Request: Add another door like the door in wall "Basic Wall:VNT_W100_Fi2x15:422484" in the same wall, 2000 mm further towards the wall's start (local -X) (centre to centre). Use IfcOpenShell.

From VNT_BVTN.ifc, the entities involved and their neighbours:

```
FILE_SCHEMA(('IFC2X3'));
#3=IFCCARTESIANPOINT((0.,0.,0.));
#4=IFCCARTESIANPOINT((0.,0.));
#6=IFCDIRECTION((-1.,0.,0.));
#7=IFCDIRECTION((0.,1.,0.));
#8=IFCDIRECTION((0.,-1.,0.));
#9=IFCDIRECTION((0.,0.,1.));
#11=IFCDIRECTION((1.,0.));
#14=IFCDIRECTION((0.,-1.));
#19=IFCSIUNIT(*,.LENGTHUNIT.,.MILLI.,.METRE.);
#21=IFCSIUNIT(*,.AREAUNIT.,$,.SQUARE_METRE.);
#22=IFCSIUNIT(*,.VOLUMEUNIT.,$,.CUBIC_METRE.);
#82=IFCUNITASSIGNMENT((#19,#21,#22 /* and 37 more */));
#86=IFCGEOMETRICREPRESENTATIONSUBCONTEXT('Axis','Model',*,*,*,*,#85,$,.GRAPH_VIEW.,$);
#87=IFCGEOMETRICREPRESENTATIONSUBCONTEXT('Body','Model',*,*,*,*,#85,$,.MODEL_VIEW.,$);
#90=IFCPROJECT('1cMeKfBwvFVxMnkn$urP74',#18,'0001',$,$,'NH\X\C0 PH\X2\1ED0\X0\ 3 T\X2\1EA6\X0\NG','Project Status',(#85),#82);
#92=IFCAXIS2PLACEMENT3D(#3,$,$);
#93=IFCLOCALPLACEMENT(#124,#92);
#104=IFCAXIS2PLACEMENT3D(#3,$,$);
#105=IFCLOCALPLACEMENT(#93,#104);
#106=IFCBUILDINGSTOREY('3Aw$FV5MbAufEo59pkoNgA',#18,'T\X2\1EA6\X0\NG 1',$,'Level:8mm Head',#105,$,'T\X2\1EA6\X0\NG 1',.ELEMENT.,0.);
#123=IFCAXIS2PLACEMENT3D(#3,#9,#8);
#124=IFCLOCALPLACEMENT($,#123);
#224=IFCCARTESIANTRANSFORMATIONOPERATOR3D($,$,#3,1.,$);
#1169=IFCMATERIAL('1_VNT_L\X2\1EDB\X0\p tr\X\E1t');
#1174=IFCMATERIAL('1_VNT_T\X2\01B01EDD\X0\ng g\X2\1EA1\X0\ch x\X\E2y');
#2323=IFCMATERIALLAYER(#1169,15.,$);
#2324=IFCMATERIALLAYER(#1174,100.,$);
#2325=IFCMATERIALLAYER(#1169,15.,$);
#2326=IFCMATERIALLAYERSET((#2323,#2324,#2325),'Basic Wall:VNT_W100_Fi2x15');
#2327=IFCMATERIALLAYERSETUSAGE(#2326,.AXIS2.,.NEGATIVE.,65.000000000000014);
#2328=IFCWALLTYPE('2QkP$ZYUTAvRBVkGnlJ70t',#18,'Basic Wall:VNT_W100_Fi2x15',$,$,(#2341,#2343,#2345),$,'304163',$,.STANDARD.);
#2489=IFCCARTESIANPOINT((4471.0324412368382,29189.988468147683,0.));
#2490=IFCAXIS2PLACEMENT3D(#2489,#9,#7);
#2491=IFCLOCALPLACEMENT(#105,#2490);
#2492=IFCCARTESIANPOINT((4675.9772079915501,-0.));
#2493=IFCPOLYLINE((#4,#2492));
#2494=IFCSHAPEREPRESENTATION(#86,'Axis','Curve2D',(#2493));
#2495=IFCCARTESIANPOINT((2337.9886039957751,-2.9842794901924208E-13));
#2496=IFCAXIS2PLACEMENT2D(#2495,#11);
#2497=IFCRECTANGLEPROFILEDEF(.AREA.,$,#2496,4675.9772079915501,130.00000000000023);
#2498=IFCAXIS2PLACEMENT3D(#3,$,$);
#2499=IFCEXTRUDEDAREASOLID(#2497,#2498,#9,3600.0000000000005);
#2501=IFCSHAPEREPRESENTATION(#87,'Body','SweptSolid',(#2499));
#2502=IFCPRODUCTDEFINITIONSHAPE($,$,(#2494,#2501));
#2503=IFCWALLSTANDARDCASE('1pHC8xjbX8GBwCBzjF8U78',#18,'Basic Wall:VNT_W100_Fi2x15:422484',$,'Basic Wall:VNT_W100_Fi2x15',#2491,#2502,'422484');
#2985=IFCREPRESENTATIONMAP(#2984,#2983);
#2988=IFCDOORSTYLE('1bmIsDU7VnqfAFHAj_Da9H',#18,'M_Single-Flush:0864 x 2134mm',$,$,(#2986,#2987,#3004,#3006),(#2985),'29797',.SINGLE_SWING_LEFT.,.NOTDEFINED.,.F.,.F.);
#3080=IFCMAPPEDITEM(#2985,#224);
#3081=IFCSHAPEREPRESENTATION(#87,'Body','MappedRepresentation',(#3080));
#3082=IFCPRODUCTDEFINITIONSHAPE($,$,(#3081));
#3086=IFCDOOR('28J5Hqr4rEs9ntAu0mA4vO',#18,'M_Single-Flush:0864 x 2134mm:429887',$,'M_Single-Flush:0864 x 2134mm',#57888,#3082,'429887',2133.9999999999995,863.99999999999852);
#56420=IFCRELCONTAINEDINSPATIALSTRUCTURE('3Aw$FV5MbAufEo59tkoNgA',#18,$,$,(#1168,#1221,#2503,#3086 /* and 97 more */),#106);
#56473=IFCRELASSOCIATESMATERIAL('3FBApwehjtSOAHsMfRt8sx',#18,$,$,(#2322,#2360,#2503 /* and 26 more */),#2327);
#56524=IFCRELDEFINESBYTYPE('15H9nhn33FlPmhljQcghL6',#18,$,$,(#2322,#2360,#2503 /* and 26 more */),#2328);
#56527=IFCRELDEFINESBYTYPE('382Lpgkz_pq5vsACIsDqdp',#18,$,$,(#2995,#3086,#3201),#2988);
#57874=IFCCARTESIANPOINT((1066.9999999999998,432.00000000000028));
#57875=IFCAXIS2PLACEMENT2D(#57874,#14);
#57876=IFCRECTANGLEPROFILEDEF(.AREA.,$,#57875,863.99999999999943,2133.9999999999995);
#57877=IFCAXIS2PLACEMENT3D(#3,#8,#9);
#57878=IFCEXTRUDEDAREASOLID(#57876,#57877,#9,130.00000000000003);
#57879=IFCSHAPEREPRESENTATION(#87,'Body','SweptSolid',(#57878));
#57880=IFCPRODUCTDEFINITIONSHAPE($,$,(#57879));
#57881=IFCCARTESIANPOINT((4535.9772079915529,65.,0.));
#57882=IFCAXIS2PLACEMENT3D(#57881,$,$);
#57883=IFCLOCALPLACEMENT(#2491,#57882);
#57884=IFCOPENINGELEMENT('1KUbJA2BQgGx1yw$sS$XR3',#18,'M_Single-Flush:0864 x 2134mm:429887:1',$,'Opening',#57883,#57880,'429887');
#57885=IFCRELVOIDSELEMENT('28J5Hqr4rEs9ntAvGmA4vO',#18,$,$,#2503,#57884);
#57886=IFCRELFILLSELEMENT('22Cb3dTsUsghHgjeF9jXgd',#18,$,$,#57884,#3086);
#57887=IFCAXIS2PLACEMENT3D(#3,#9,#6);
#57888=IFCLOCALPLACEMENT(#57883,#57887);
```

```python
import ifcopenshell
import ifcopenshell.api.feature
import ifcopenshell.api.geometry
import ifcopenshell.api.root
import ifcopenshell.geom
import ifcopenshell.util.element
import ifcopenshell.util.placement
import ifcopenshell.util.shape

model = ifcopenshell.open("VNT_BVTN.ifc")
settings = ifcopenshell.geom.settings()


def volume(element):
    """Net volume in cubic metres, openings subtracted."""
    shape = ifcopenshell.geom.create_shape(settings, element)
    return ifcopenshell.util.shape.get_volume(shape.geometry)


def reuse_history(source, copy):
    """copy_class also copies each property set's owner history, people and application; keep the originals."""
    for rel in copy.IsDefinedBy:
        if rel.is_a("IfcRelDefinesByProperties") and (history := rel.RelatingPropertyDefinition.OwnerHistory):
            rel.RelatingPropertyDefinition.OwnerHistory = source.OwnerHistory
            ifcopenshell.util.element.remove_deep2(model, history)


door = model.by_guid("28J5Hqr4rEs9ntAu0mA4vO")
opening = door.FillsVoids[0].RelatingOpeningElement
wall = opening.VoidsElements[0].RelatingBuildingElement
before = volume(wall)
shift = ifcopenshell.util.placement.get_local_placement(wall.ObjectPlacement)[:3, 0] * -2000.0

# copy_class copies the void relationship, type, container and properties, but no geometry.
new_opening = ifcopenshell.api.root.copy_class(model, product=opening)
new_opening.Representation = ifcopenshell.util.element.copy_deep(
    model, opening.Representation, exclude=["IfcGeometricRepresentationContext", "IfcRepresentationMap"]
)
new_opening.Name = "M_Single-Flush:0864 x 2134mm"
new_opening.Tag = None
new_door = ifcopenshell.api.root.copy_class(model, product=door)
new_door.Representation = ifcopenshell.util.element.copy_deep(
    model, door.Representation, exclude=["IfcGeometricRepresentationContext", "IfcRepresentationMap"]
)
new_door.Name = "M_Single-Flush:0864 x 2134mm"
new_door.Tag = None
reuse_history(door, new_door)
fills = ifcopenshell.api.feature.add_filling(model, opening=new_opening, element=new_door)
fills.OwnerHistory = new_door.OwnerHistory  # required in IFC2X3

for old, new in ((opening, new_opening), (door, new_door)):
    matrix = ifcopenshell.util.placement.get_local_placement(old.ObjectPlacement)
    matrix[:3, 3] += shift
    ifcopenshell.api.geometry.edit_object_placement(model, product=new, matrix=matrix, is_si=False)

after = volume(wall)

print(f"wall volume {before:.3f} -> {after:.3f} m3")

model.write("VNT_BVTN_rev.ifc")
```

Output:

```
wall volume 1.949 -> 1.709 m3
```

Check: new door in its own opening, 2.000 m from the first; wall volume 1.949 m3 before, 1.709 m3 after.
